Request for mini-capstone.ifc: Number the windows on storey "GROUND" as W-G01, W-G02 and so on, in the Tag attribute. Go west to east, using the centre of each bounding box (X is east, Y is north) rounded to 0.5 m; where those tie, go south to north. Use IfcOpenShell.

First a look at what the model holds.

```python
import ifcopenshell
import ifcopenshell.util.element
import ifcopenshell.util.placement

model = ifcopenshell.open("mini-capstone.ifc")
print(model.schema)
storey = next(s for s in model.by_type("IfcBuildingStorey") if s.Name == "GROUND")
windows = [e for e in ifcopenshell.util.element.get_decomposition(storey) if e.is_a("IfcWindow")]
for e in sorted(windows, key=lambda e: e.id()):
    origin = ifcopenshell.util.placement.get_local_placement(e.ObjectPlacement)[:3, 3]
    print(e.id(), e.Tag, e.Name, origin.round(2) + 0.0, sep=" | ")
```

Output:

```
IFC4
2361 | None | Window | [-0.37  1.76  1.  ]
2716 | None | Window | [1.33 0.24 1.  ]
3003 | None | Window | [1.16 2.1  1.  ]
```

```python
import ifcopenshell
import ifcopenshell.geom
import ifcopenshell.util.element
import ifcopenshell.util.shape

model = ifcopenshell.open("mini-capstone.ifc")
settings = ifcopenshell.geom.settings()
settings.set("use-world-coords", True)


def centre(element):
    shape = ifcopenshell.geom.create_shape(settings, element)
    return ifcopenshell.util.shape.get_bbox_centroid(shape.geometry)


storey = next(s for s in model.by_type("IfcBuildingStorey") if s.Name == "GROUND")
windows = [e for e in ifcopenshell.util.element.get_decomposition(storey) if e.is_a("IfcWindow")]

# Insertion points can sit at a corner or the storey origin, so sort by the geometry (in metres).
centres = {e: centre(e) for e in windows}
windows.sort(key=lambda e: (round(centres[e][0] / 0.5), centres[e][1]))

for i, e in enumerate(windows, start=1):
    number = f"W-G{i:02d}"
    e.Tag = number
    print(e.id(), number)

model.write("mini-capstone-out.ifc")
```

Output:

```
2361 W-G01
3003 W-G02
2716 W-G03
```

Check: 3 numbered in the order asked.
